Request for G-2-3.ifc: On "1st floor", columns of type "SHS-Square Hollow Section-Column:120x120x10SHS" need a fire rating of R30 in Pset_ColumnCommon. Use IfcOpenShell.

First a look at what the model holds.

```python
import ifcopenshell
import ifcopenshell.util.element

model = ifcopenshell.open("G-2-3.ifc")
print(model.schema)
storey = next(s for s in model.by_type("IfcBuildingStorey") if s.Name == "1st floor")
columns = [e for e in ifcopenshell.util.element.get_decomposition(storey) if e.is_a("IfcColumn")]
seen = {}
for e in columns:
    element_type = ifcopenshell.util.element.get_type(e)
    key = (element_type.Name if element_type != e and element_type else None, ifcopenshell.util.element.get_pset(e, "Pset_ColumnCommon", "FireRating"))
    seen[key] = seen.get(key, 0) + 1
for (name, value), count in sorted(seen.items(), key=str):
    print(count, "x", name, "|", value)
```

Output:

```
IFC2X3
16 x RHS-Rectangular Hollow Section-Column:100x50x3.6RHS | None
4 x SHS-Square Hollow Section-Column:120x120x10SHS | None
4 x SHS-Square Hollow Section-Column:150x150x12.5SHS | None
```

```python
import ifcopenshell
import ifcopenshell.api.pset
import ifcopenshell.util.element

model = ifcopenshell.open("G-2-3.ifc")

storey = next(s for s in model.by_type("IfcBuildingStorey") if s.Name == "1st floor")
columns = [e for e in ifcopenshell.util.element.get_decomposition(storey) if e.is_a("IfcColumn")]

count = 0
for e in columns:
    element_type = ifcopenshell.util.element.get_type(e)
    if element_type in (None, e) or element_type.Name != "SHS-Square Hollow Section-Column:120x120x10SHS":
        continue
    # add_pset returns the element's existing set when there is one.
    pset = ifcopenshell.api.pset.add_pset(model, product=e, name="Pset_ColumnCommon")
    ifcopenshell.api.pset.edit_pset(model, pset=pset, properties={"FireRating": "R30"})
    count += 1

print(count, "columns updated")

model.write("G-2-3_updated.ifc")
```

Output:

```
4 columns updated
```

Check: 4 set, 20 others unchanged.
